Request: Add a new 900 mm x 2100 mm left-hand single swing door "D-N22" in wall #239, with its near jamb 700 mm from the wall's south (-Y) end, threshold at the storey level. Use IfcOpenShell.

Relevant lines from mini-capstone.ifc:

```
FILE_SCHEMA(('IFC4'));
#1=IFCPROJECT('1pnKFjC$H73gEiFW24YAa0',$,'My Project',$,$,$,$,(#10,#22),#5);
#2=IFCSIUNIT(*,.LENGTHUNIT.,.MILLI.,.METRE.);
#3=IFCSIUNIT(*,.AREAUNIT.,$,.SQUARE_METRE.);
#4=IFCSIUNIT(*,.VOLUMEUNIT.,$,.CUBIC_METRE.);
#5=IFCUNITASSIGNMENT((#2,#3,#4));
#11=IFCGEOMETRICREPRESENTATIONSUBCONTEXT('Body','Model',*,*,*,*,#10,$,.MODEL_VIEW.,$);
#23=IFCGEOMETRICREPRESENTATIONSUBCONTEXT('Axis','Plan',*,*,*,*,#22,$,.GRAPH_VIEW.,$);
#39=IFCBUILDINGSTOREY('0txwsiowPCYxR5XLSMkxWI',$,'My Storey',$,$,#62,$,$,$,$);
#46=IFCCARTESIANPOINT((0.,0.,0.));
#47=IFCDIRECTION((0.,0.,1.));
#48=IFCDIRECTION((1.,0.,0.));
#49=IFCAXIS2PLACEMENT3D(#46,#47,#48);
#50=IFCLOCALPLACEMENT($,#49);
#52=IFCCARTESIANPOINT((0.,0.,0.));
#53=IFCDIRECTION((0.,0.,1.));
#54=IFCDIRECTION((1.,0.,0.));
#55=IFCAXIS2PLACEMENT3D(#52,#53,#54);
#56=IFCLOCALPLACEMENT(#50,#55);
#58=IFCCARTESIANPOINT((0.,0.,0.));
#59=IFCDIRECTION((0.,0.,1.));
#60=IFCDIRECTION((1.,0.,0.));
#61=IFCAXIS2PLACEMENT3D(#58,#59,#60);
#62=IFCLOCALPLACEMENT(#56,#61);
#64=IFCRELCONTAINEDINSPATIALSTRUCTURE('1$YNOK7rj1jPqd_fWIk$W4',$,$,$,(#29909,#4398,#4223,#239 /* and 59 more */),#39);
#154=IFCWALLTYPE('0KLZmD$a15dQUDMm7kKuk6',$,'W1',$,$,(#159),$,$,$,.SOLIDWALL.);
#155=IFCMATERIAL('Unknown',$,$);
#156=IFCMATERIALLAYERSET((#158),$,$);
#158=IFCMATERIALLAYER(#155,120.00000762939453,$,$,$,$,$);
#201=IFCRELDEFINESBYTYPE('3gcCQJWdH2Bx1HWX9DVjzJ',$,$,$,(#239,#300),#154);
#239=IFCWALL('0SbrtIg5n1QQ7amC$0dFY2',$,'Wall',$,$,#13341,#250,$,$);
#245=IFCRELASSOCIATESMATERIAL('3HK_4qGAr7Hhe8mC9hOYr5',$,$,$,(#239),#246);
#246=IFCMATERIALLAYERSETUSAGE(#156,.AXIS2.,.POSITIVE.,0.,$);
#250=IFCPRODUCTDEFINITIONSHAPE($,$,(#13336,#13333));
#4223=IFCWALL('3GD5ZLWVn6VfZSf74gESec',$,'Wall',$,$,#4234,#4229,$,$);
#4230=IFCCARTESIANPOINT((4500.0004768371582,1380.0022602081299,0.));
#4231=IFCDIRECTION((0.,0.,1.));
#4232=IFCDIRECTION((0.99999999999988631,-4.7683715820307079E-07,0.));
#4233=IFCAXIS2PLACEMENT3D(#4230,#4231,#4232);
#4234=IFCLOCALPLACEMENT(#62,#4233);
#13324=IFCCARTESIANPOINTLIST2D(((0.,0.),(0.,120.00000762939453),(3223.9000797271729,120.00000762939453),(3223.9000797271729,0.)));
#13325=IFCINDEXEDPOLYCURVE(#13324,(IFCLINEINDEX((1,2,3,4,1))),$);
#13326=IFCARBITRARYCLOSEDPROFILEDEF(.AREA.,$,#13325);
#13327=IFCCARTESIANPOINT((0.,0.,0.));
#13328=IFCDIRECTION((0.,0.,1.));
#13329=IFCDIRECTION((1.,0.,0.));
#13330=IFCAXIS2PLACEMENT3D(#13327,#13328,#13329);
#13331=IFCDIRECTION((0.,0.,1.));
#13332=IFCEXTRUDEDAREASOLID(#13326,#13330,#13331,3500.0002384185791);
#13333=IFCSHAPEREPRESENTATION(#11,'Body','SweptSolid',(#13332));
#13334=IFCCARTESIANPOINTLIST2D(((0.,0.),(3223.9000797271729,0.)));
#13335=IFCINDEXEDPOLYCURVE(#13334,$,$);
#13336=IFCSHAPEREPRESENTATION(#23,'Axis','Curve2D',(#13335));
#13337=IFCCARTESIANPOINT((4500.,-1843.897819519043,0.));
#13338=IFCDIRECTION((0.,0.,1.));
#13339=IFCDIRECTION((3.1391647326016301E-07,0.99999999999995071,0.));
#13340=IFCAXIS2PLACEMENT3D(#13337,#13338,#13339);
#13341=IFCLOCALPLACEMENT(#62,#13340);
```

```python
import numpy as np
import ifcopenshell
import ifcopenshell.api.feature
import ifcopenshell.api.geometry
import ifcopenshell.api.root
import ifcopenshell.api.spatial
import ifcopenshell.geom
import ifcopenshell.util.element
import ifcopenshell.util.placement
import ifcopenshell.util.representation
import ifcopenshell.util.shape
import ifcopenshell.util.unit

model = ifcopenshell.open("mini-capstone.ifc")
unit_scale = ifcopenshell.util.unit.calculate_unit_scale(model)
settings = ifcopenshell.geom.settings()


def volume(element):
    """Net volume in cubic metres, openings subtracted."""
    shape = ifcopenshell.geom.create_shape(settings, element)
    return ifcopenshell.util.shape.get_volume(shape.geometry)


wall = model.by_id(239)
storey = ifcopenshell.util.element.get_container(wall, ifc_class="IfcBuildingStorey")
context = ifcopenshell.util.representation.get_context(model, "Model", "Body", "MODEL_VIEW")
before = volume(wall)

width, height, from_end, sill = 0.9, 2.1, 0.7, 0.0  # metres

# The wall runs along its own X axis, and the end named is its -X end.
wall_shape = ifcopenshell.geom.create_shape(settings, wall)
x, y, z = ifcopenshell.util.shape.get_vertices(wall_shape.geometry).T
start = x.min() + from_end
face, thickness = float(y.min()), float(y.max() - y.min())
wall_matrix = ifcopenshell.util.placement.get_local_placement(wall.ObjectPlacement)
level = ifcopenshell.util.placement.get_local_placement(storey.ObjectPlacement)[2, 3]


def in_wall(x, y):
    """Placement at x, y metres in the wall's axes, at sill height."""
    matrix = wall_matrix.copy()
    matrix[:, 3] = wall_matrix @ np.array([x / unit_scale, y / unit_scale, 0.0, 1.0])
    matrix[2, 3] = level + sill / unit_scale
    return matrix


# Opening: a box that overshoots both wall faces by 50 mm.
opening = ifcopenshell.api.root.create_entity(model, ifc_class="IfcOpeningElement", predefined_type="OPENING")
box = ifcopenshell.api.geometry.add_wall_representation(
    model, context=context, length=width, height=height, thickness=thickness + 0.1
)
ifcopenshell.api.geometry.assign_representation(model, product=opening, representation=box)
ifcopenshell.api.geometry.edit_object_placement(model, product=opening, matrix=in_wall(start, face - 0.05), is_si=False)
ifcopenshell.api.feature.add_feature(model, feature=opening, element=wall)

door = ifcopenshell.api.root.create_entity(model, ifc_class="IfcDoor", name="D-N22", predefined_type="DOOR")
door.OverallWidth, door.OverallHeight = width / unit_scale, height / unit_scale
door.OperationType = "SINGLE_SWING_LEFT"
body = ifcopenshell.api.geometry.add_door_representation(
    model,
    context=context,
    overall_width=door.OverallWidth,
    overall_height=door.OverallHeight,
    operation_type="SINGLE_SWING_LEFT",
    lining_properties={"LiningDepth": thickness / unit_scale, "ThresholdDepth": thickness / unit_scale},
)
ifcopenshell.api.geometry.assign_representation(model, product=door, representation=body)
ifcopenshell.api.spatial.assign_container(model, products=[door], relating_structure=storey)
ifcopenshell.api.feature.add_filling(model, opening=opening, element=door)

# The lining spans the wall, so the door starts at the wall face.
ifcopenshell.api.geometry.edit_object_placement(model, product=door, matrix=in_wall(start, face), is_si=False)

after = volume(wall)

print(f"wall volume {before:.3f} -> {after:.3f} m3")

model.write("mini-capstone-out.ifc")
```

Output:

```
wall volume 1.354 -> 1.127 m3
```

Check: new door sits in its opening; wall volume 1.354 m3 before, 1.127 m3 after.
